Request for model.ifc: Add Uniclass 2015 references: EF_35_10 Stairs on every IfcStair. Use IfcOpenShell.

First a look at what the model holds.

```python
import ifcopenshell

model = ifcopenshell.open("model.ifc")
print(model.schema)
print("classifications:", [c.Name for c in model.by_type("IfcClassification")])
for ifc_class in ("IfcDoor", "IfcRoof", "IfcStair", "IfcWall", "IfcWindow"):
    print(ifc_class, len(model.by_type(ifc_class)))
```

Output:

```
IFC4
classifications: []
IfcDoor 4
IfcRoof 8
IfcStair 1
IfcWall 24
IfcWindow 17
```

```python
import ifcopenshell
import ifcopenshell.api.classification

model = ifcopenshell.open("model.ifc")

system = ifcopenshell.api.classification.add_classification(model, classification="Uniclass 2015")

codes = {
    "IfcStair": ("EF_35_10", "Stairs"),
}
for ifc_class, (code, name) in codes.items():
    products = model.by_type(ifc_class)
    ifcopenshell.api.classification.add_reference(
        model, products=products, classification=system, identification=code, name=name
    )
    print(code, len(products))

model.write("model_rev.ifc")
```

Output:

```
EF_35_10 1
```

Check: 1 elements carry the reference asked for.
